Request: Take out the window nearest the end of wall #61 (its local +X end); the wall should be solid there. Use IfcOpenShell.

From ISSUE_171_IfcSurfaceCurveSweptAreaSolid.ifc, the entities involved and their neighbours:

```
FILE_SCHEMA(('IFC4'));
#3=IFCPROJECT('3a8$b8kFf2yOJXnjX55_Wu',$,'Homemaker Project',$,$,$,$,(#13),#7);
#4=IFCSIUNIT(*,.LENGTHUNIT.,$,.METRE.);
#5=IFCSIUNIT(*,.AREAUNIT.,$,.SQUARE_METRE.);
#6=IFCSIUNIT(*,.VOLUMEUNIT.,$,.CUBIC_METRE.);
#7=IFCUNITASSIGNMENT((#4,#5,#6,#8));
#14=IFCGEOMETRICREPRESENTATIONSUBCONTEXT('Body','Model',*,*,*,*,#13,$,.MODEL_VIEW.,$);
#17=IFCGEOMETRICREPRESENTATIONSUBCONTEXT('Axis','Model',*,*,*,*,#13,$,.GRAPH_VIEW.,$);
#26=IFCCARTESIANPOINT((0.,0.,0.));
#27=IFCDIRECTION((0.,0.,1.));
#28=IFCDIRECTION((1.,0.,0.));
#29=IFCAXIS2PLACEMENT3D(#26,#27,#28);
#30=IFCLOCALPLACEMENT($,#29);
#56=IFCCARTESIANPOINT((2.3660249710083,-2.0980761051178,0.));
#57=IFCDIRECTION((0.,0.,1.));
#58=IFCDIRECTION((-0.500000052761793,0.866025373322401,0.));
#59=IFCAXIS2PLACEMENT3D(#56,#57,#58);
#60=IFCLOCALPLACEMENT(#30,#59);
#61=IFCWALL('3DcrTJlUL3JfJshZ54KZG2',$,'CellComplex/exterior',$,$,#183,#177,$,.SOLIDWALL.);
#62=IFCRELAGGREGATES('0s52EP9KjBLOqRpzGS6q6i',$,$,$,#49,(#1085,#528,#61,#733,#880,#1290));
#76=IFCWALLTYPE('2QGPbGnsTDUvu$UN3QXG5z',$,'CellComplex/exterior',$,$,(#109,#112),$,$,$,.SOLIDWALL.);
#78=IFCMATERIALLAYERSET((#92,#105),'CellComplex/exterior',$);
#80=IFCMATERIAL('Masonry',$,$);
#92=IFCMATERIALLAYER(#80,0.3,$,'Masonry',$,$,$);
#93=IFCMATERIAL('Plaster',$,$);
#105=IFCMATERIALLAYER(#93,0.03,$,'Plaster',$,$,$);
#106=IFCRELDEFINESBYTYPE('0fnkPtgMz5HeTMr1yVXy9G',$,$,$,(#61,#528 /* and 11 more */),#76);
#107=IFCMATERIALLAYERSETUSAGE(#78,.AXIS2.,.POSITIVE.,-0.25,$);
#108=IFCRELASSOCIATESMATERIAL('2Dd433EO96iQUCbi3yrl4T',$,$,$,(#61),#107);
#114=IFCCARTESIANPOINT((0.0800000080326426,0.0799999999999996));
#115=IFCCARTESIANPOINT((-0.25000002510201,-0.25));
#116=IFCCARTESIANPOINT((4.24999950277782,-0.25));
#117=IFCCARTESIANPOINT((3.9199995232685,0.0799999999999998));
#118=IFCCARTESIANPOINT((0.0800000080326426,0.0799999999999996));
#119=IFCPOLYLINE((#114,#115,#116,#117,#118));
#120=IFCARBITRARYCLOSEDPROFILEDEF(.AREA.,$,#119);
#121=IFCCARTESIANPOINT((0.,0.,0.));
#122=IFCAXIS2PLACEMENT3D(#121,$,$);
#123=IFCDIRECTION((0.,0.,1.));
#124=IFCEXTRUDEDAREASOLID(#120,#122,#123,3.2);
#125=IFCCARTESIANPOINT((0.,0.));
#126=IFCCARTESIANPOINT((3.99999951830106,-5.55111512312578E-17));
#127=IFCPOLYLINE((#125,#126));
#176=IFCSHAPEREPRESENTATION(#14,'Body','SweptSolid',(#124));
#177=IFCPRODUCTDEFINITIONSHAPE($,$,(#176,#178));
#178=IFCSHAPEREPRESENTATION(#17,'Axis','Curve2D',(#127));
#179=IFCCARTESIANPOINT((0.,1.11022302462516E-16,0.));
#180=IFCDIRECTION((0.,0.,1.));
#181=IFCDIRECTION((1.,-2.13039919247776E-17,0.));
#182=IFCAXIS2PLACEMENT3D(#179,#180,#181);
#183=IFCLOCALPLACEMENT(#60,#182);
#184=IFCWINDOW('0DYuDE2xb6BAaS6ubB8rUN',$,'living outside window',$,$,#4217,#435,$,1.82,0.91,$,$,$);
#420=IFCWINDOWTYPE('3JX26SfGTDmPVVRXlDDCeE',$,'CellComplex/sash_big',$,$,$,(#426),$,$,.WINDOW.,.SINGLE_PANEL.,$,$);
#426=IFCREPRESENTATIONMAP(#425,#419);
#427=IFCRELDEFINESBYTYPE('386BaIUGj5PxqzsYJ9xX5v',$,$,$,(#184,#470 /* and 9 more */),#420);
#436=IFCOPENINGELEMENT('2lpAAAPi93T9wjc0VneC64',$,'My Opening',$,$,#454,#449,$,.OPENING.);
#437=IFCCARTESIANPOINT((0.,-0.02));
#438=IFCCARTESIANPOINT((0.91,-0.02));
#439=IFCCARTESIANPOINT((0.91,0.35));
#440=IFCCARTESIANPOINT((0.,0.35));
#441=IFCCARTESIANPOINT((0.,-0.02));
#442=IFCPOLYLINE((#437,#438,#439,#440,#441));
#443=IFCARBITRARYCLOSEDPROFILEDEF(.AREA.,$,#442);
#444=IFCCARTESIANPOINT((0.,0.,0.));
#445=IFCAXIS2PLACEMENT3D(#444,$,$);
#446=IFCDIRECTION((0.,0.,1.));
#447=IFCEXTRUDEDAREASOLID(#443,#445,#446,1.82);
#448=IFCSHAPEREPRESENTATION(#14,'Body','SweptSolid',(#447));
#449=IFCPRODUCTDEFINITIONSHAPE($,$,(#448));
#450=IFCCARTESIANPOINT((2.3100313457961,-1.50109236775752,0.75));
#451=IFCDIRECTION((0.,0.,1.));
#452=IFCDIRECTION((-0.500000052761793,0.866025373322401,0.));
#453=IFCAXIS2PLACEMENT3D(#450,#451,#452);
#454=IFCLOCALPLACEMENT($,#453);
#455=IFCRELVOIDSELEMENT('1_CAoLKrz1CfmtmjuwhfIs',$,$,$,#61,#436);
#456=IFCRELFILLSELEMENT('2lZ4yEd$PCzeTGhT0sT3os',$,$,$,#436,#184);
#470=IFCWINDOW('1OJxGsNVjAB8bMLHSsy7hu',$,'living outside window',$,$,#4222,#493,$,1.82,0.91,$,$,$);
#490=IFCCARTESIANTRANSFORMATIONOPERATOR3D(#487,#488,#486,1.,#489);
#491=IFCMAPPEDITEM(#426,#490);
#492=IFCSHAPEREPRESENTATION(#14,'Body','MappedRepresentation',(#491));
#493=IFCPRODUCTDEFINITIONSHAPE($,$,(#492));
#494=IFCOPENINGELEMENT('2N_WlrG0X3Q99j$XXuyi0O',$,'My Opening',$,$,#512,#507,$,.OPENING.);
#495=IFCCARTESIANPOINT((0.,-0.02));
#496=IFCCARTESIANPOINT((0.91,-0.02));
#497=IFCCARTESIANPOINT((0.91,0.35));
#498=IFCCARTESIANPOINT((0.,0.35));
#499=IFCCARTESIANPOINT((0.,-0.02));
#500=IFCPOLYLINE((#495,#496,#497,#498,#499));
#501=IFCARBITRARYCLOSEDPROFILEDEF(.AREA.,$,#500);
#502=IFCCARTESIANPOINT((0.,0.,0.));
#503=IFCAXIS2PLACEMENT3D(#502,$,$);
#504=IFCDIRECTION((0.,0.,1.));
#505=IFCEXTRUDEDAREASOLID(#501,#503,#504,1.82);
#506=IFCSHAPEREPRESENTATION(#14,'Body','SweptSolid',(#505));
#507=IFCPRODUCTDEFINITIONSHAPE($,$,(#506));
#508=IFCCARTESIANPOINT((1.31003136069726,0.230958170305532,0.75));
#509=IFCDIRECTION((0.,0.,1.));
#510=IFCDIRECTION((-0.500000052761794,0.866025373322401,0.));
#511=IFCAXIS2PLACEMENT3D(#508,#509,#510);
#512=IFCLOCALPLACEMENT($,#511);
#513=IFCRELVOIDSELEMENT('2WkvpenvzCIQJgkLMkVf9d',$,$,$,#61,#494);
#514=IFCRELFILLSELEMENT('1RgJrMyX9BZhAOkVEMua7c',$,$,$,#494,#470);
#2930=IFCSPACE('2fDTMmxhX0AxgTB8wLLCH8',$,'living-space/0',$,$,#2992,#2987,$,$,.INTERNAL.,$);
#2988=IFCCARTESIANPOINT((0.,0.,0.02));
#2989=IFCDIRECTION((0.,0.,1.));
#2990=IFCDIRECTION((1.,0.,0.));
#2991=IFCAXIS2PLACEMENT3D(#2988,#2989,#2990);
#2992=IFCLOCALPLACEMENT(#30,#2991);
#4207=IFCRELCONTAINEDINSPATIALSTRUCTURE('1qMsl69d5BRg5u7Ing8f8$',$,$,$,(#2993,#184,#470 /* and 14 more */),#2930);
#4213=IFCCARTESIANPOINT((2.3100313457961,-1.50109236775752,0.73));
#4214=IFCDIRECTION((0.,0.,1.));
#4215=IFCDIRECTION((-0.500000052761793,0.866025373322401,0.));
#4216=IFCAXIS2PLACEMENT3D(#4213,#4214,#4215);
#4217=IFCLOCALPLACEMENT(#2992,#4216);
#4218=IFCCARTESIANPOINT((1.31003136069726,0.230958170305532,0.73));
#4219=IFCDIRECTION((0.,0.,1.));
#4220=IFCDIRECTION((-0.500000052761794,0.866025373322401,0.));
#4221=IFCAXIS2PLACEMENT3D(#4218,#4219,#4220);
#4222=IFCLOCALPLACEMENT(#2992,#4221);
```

```python
import ifcopenshell
import ifcopenshell.api.feature
import ifcopenshell.api.root
import ifcopenshell.geom
import ifcopenshell.util.shape

model = ifcopenshell.open("ISSUE_171_IfcSurfaceCurveSweptAreaSolid.ifc")
settings = ifcopenshell.geom.settings()


def volume(element):
    """Net volume in cubic metres, openings subtracted."""
    shape = ifcopenshell.geom.create_shape(settings, element)
    return ifcopenshell.util.shape.get_volume(shape.geometry)


window = model.by_id(470)
opening = window.FillsVoids[0].RelatingOpeningElement
wall = opening.VoidsElements[0].RelatingBuildingElement
before = volume(wall)

ifcopenshell.api.root.remove_product(model, product=window)
ifcopenshell.api.feature.remove_feature(model, feature=opening)

after = volume(wall)

print(f"wall volume {before:.3f} -> {after:.3f} m3")

model.write("ISSUE_171_IfcSurfaceCurveSweptAreaSolid_v2.ifc")
```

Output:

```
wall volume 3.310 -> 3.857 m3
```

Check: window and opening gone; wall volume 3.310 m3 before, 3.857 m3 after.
